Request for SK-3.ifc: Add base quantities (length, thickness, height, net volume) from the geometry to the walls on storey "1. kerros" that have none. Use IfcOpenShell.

First a look at what the model holds.

```python
import ifcopenshell
import ifcopenshell.util.element
import ifcopenshell.util.unit

model = ifcopenshell.open("SK-3.ifc")
print(model.schema)
for unit_type in ("LENGTHUNIT", "AREAUNIT", "VOLUMEUNIT"):
    print(unit_type, ifcopenshell.util.unit.calculate_unit_scale(model, unit_type))
storey = next(s for s in model.by_type("IfcBuildingStorey") if s.Name == "1. kerros")
walls = [e for e in ifcopenshell.util.element.get_decomposition(storey) if e.is_a("IfcWall")]
for e in sorted(walls, key=lambda e: e.id()):
    print(e.id(), e.is_a(), e.Name, list(ifcopenshell.util.element.get_psets(e, qtos_only=True)), sep=" | ")
```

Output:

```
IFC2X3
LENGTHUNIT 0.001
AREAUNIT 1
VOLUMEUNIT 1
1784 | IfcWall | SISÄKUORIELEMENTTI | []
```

```python
import ifcopenshell
import ifcopenshell.api.pset
import ifcopenshell.geom
import ifcopenshell.util.element
import ifcopenshell.util.shape
import ifcopenshell.util.unit

model = ifcopenshell.open("SK-3.ifc")
unit_scale = ifcopenshell.util.unit.calculate_unit_scale(model)
volume_scale = ifcopenshell.util.unit.calculate_unit_scale(model, "VOLUMEUNIT")
settings = ifcopenshell.geom.settings()

storey = next(s for s in model.by_type("IfcBuildingStorey") if s.Name == "1. kerros")
walls = [e for e in ifcopenshell.util.element.get_decomposition(storey) if e.is_a("IfcWall")]

for e in sorted(walls, key=lambda e: e.id()):
    if ifcopenshell.util.element.get_psets(e, qtos_only=True, should_inherit=False):
        continue
    # Geometry comes back in metres, in the element's own axes.
    shape = ifcopenshell.geom.create_shape(settings, e)
    values = {
        "Length": ifcopenshell.util.shape.get_x(shape.geometry) / unit_scale,
        "Width": ifcopenshell.util.shape.get_y(shape.geometry) / unit_scale,
        "Height": ifcopenshell.util.shape.get_z(shape.geometry) / unit_scale,
        "NetVolume": ifcopenshell.util.shape.get_volume(shape.geometry) / volume_scale,
    }
    qto = ifcopenshell.api.pset.add_qto(model, product=e, name="BaseQuantities")
    ifcopenshell.api.pset.edit_qto(model, qto=qto, properties=values)
    print(e.id(), {k: round(v, 3) for k, v in values.items()})

model.write("SK-3-out.ifc")
```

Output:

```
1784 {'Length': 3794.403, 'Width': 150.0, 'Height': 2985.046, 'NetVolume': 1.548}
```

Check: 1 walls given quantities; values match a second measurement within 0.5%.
